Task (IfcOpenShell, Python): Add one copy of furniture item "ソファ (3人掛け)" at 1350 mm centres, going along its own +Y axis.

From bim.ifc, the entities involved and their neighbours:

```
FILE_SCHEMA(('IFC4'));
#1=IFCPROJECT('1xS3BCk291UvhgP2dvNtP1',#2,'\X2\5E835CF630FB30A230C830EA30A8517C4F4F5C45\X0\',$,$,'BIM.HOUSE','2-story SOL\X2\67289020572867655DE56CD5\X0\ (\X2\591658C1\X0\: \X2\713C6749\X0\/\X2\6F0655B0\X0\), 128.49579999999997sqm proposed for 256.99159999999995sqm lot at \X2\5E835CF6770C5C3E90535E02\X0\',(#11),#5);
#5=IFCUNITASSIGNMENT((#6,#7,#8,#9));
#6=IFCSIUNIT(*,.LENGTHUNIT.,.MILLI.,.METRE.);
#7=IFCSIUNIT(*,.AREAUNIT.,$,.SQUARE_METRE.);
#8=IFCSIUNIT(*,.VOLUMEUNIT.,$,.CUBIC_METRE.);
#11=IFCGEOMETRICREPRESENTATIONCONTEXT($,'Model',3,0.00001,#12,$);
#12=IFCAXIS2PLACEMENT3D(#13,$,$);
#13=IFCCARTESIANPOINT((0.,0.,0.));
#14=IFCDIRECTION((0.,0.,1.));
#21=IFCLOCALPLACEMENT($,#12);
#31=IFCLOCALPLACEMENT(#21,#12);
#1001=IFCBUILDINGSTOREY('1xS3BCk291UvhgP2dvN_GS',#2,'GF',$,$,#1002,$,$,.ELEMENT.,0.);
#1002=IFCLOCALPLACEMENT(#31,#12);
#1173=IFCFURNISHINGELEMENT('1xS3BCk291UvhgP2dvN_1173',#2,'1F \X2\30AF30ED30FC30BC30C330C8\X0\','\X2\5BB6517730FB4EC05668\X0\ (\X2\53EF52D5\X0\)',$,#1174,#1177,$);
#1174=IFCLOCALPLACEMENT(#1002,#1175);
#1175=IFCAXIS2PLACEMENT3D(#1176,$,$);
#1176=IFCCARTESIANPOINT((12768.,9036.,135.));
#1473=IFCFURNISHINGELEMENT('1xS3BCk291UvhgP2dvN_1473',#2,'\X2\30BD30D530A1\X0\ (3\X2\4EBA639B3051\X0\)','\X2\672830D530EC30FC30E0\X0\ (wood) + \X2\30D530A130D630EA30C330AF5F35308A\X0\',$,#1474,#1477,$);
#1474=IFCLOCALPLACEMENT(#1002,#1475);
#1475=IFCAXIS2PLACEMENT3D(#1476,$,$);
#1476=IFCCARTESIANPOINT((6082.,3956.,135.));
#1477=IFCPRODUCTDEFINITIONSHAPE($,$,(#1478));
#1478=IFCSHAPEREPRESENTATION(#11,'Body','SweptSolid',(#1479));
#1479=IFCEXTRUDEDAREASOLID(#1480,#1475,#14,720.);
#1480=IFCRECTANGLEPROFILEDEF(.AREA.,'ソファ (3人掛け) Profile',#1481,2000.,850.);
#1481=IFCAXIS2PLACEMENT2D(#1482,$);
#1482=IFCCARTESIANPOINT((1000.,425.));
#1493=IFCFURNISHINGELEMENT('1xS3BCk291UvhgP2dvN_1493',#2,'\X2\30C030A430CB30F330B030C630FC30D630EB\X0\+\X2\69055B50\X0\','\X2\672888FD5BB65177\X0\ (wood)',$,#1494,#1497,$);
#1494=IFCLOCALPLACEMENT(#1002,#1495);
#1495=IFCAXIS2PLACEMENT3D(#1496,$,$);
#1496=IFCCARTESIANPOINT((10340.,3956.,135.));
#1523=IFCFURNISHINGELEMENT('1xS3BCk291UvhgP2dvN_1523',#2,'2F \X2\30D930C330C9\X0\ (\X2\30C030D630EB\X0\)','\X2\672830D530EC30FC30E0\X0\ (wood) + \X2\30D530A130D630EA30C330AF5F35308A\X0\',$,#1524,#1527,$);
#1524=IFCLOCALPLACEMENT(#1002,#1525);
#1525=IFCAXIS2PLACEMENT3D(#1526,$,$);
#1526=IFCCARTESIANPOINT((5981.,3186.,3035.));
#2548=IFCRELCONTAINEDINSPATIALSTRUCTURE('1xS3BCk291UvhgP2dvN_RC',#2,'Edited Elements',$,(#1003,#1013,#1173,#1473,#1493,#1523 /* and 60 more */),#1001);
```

```python
import ifcopenshell
import ifcopenshell.api.geometry
import ifcopenshell.api.root
import ifcopenshell.util.element
import ifcopenshell.util.placement
import ifcopenshell.util.unit

model = ifcopenshell.open("bim.ifc")
unit_scale = ifcopenshell.util.unit.calculate_unit_scale(model)


def reuse_history(source, copy):
    """copy_class also copies each property set's owner history, people and application; keep the originals."""
    for rel in copy.IsDefinedBy:
        if rel.is_a("IfcRelDefinesByProperties") and (history := rel.RelatingPropertyDefinition.OwnerHistory):
            rel.RelatingPropertyDefinition.OwnerHistory = source.OwnerHistory
            ifcopenshell.util.element.remove_deep2(model, history)


source = model.by_guid("1xS3BCk291UvhgP2dvN_1473")
base = ifcopenshell.util.placement.get_local_placement(source.ObjectPlacement)
step = base[:3, 1] * 1.35 / unit_scale

for i in range(1, 2):
    copy = ifcopenshell.api.root.copy_class(model, product=source)
    copy.Representation = ifcopenshell.util.element.copy_deep(
        model, source.Representation, exclude=["IfcGeometricRepresentationContext", "IfcRepresentationMap"]
    )
    reuse_history(source, copy)
    matrix = base.copy()
    matrix[:3, 3] += i * step
    print("added at", matrix[:3, 3].round(3) + 0.0)
    ifcopenshell.api.geometry.edit_object_placement(model, product=copy, matrix=matrix, is_si=False)

model.write("bim_updated.ifc")
```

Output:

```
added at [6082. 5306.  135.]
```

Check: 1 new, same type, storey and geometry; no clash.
